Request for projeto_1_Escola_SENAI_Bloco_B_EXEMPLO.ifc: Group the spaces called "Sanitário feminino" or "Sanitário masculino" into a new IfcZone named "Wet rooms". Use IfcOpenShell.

First a look at what the model holds.

```python
import ifcopenshell

model = ifcopenshell.open("projeto_1_Escola_SENAI_Bloco_B_EXEMPLO.ifc")
print(model.schema)
seen = {}
for space in model.by_type("IfcSpace"):
    seen[space.LongName] = seen.get(space.LongName, 0) + 1
for name, count in sorted(seen.items(), key=str):
    print(count, "x", name)
print("zones:", [z.Name for z in model.by_type("IfcZone")][:20])
```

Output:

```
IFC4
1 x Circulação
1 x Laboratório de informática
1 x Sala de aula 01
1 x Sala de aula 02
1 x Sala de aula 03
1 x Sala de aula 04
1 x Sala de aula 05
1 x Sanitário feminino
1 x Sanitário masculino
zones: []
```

```python
import ifcopenshell
import ifcopenshell.api.group
import ifcopenshell.api.root

model = ifcopenshell.open("projeto_1_Escola_SENAI_Bloco_B_EXEMPLO.ifc")

names = {"Sanitário feminino", "Sanitário masculino"}
spaces = [s for s in model.by_type("IfcSpace") if s.LongName in names]

zone = ifcopenshell.api.root.create_entity(model, ifc_class="IfcZone", name="Wet rooms")
ifcopenshell.api.group.assign_group(model, products=spaces, group=zone)
print(len(spaces), "spaces in", zone.Name)

model.write("projeto_1_Escola_SENAI_Bloco_B_EXEMPLO_updated.ifc")
```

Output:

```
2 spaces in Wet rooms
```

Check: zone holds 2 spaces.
